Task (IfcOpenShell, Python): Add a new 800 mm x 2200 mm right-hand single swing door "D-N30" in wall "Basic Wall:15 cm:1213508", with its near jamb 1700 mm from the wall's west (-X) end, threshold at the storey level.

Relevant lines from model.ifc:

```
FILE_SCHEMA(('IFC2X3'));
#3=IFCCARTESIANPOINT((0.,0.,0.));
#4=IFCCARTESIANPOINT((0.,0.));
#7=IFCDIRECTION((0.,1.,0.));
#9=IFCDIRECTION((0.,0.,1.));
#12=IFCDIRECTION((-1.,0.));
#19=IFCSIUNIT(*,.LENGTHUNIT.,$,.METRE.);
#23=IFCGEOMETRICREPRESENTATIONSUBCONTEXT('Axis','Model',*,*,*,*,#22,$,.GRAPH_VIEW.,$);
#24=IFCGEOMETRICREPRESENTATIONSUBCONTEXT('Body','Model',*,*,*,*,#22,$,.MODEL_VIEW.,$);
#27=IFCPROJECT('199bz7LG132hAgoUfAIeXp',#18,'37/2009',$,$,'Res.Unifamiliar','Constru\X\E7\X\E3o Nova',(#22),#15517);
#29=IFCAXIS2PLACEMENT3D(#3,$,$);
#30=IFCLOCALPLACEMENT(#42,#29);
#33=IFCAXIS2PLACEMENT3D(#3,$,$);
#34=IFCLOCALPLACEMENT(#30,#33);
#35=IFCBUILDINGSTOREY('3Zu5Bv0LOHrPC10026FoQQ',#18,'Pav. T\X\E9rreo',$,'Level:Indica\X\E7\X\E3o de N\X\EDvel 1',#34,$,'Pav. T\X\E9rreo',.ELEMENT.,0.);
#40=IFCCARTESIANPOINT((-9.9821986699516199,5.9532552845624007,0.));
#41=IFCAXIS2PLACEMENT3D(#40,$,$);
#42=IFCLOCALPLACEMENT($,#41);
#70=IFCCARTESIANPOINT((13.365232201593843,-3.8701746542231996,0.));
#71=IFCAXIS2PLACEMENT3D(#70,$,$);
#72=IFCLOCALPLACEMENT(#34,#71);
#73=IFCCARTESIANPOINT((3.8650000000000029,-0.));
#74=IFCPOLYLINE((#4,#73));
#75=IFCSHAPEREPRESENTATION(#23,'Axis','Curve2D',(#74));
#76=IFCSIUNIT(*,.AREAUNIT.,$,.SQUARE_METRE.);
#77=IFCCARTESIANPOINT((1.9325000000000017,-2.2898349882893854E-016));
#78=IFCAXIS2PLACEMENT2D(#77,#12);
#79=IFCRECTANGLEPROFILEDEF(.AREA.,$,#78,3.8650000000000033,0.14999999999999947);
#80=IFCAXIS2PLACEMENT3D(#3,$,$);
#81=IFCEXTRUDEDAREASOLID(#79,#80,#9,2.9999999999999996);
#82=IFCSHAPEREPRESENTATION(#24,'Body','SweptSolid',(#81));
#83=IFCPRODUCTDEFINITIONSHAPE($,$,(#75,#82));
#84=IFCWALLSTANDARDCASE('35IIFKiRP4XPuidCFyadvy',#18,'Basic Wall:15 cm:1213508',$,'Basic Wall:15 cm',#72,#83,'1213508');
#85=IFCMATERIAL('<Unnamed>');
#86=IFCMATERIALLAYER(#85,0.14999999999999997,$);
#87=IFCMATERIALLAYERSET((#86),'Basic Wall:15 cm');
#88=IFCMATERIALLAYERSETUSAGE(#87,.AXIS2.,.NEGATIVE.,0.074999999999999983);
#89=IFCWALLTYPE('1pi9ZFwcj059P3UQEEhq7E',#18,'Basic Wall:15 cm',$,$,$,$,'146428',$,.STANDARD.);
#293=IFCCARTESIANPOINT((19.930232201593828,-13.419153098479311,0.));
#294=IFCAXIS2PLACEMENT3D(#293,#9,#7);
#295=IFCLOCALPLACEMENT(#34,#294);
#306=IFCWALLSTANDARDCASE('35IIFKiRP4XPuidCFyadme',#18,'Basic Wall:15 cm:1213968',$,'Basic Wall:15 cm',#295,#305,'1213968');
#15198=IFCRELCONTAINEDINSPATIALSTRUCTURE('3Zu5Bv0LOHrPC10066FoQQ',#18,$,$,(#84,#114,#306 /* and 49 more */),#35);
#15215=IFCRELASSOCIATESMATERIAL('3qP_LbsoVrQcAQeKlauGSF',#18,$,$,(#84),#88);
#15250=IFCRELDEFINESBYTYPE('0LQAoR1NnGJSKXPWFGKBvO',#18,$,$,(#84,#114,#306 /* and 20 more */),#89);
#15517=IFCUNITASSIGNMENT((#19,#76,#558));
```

```python
import numpy as np
import ifcopenshell
import ifcopenshell.api.feature
import ifcopenshell.api.geometry
import ifcopenshell.api.root
import ifcopenshell.api.spatial
import ifcopenshell.api.type
import ifcopenshell.geom
import ifcopenshell.util.element
import ifcopenshell.util.placement
import ifcopenshell.util.representation
import ifcopenshell.util.shape
import ifcopenshell.util.unit

model = ifcopenshell.open("model.ifc")
unit_scale = ifcopenshell.util.unit.calculate_unit_scale(model)
settings = ifcopenshell.geom.settings()


def volume(element):
    """Net volume in cubic metres, openings subtracted."""
    shape = ifcopenshell.geom.create_shape(settings, element)
    return ifcopenshell.util.shape.get_volume(shape.geometry)


wall = model.by_id(84)
storey = ifcopenshell.util.element.get_container(wall, ifc_class="IfcBuildingStorey")
context = ifcopenshell.util.representation.get_context(model, "Model", "Body", "MODEL_VIEW")
before = volume(wall)

width, height, from_end, sill = 0.8, 2.2, 1.7, 0.0  # metres

# The wall runs along its own X axis, and the end named is its -X end.
wall_shape = ifcopenshell.geom.create_shape(settings, wall)
x, y, z = ifcopenshell.util.shape.get_vertices(wall_shape.geometry).T
start = x.min() + from_end
face, thickness = float(y.min()), float(y.max() - y.min())
wall_matrix = ifcopenshell.util.placement.get_local_placement(wall.ObjectPlacement)
level = ifcopenshell.util.placement.get_local_placement(storey.ObjectPlacement)[2, 3]


def in_wall(x, y):
    """Placement at x, y metres in the wall's axes, at sill height."""
    matrix = wall_matrix.copy()
    matrix[:, 3] = wall_matrix @ np.array([x / unit_scale, y / unit_scale, 0.0, 1.0])
    matrix[2, 3] = level + sill / unit_scale
    return matrix


# Opening: a box that overshoots both wall faces by 50 mm.
opening = ifcopenshell.api.root.create_entity(model, ifc_class="IfcOpeningElement")
box = ifcopenshell.api.geometry.add_wall_representation(
    model, context=context, length=width, height=height, thickness=thickness + 0.1
)
ifcopenshell.api.geometry.assign_representation(model, product=opening, representation=box)
ifcopenshell.api.geometry.edit_object_placement(model, product=opening, matrix=in_wall(start, face - 0.05), is_si=False)
ifcopenshell.api.feature.add_feature(model, feature=opening, element=wall)

door = ifcopenshell.api.root.create_entity(model, ifc_class="IfcDoor", name="D-N30")
door.OverallWidth, door.OverallHeight = width / unit_scale, height / unit_scale
body = ifcopenshell.api.geometry.add_door_representation(
    model,
    context=context,
    overall_width=door.OverallWidth,
    overall_height=door.OverallHeight,
    operation_type="SINGLE_SWING_RIGHT",
    lining_properties={"LiningDepth": thickness / unit_scale, "ThresholdDepth": thickness / unit_scale},
)
ifcopenshell.api.geometry.assign_representation(model, product=door, representation=body)
ifcopenshell.api.spatial.assign_container(model, products=[door], relating_structure=storey)
fills = ifcopenshell.api.feature.add_filling(model, opening=opening, element=door)
fills.OwnerHistory = door.OwnerHistory  # required in IFC2X3

# IFC2X3 keeps the operation on the door style.
style = ifcopenshell.api.root.create_entity(model, ifc_class="IfcDoorStyle", name="D-N30")
style.OperationType, style.ConstructionType = "SINGLE_SWING_RIGHT", "NOTDEFINED"
style.ParameterTakesPrecedence = style.Sizeable = False
ifcopenshell.api.type.assign_type(model, related_objects=[door], relating_type=style)

# The lining spans the wall, so the door starts at the wall face.
ifcopenshell.api.geometry.edit_object_placement(model, product=door, matrix=in_wall(start, face), is_si=False)

after = volume(wall)

print(f"wall volume {before:.3f} -> {after:.3f} m3")

model.write("model-out.ifc")
```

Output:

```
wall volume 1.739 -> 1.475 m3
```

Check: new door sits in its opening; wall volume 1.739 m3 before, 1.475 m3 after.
